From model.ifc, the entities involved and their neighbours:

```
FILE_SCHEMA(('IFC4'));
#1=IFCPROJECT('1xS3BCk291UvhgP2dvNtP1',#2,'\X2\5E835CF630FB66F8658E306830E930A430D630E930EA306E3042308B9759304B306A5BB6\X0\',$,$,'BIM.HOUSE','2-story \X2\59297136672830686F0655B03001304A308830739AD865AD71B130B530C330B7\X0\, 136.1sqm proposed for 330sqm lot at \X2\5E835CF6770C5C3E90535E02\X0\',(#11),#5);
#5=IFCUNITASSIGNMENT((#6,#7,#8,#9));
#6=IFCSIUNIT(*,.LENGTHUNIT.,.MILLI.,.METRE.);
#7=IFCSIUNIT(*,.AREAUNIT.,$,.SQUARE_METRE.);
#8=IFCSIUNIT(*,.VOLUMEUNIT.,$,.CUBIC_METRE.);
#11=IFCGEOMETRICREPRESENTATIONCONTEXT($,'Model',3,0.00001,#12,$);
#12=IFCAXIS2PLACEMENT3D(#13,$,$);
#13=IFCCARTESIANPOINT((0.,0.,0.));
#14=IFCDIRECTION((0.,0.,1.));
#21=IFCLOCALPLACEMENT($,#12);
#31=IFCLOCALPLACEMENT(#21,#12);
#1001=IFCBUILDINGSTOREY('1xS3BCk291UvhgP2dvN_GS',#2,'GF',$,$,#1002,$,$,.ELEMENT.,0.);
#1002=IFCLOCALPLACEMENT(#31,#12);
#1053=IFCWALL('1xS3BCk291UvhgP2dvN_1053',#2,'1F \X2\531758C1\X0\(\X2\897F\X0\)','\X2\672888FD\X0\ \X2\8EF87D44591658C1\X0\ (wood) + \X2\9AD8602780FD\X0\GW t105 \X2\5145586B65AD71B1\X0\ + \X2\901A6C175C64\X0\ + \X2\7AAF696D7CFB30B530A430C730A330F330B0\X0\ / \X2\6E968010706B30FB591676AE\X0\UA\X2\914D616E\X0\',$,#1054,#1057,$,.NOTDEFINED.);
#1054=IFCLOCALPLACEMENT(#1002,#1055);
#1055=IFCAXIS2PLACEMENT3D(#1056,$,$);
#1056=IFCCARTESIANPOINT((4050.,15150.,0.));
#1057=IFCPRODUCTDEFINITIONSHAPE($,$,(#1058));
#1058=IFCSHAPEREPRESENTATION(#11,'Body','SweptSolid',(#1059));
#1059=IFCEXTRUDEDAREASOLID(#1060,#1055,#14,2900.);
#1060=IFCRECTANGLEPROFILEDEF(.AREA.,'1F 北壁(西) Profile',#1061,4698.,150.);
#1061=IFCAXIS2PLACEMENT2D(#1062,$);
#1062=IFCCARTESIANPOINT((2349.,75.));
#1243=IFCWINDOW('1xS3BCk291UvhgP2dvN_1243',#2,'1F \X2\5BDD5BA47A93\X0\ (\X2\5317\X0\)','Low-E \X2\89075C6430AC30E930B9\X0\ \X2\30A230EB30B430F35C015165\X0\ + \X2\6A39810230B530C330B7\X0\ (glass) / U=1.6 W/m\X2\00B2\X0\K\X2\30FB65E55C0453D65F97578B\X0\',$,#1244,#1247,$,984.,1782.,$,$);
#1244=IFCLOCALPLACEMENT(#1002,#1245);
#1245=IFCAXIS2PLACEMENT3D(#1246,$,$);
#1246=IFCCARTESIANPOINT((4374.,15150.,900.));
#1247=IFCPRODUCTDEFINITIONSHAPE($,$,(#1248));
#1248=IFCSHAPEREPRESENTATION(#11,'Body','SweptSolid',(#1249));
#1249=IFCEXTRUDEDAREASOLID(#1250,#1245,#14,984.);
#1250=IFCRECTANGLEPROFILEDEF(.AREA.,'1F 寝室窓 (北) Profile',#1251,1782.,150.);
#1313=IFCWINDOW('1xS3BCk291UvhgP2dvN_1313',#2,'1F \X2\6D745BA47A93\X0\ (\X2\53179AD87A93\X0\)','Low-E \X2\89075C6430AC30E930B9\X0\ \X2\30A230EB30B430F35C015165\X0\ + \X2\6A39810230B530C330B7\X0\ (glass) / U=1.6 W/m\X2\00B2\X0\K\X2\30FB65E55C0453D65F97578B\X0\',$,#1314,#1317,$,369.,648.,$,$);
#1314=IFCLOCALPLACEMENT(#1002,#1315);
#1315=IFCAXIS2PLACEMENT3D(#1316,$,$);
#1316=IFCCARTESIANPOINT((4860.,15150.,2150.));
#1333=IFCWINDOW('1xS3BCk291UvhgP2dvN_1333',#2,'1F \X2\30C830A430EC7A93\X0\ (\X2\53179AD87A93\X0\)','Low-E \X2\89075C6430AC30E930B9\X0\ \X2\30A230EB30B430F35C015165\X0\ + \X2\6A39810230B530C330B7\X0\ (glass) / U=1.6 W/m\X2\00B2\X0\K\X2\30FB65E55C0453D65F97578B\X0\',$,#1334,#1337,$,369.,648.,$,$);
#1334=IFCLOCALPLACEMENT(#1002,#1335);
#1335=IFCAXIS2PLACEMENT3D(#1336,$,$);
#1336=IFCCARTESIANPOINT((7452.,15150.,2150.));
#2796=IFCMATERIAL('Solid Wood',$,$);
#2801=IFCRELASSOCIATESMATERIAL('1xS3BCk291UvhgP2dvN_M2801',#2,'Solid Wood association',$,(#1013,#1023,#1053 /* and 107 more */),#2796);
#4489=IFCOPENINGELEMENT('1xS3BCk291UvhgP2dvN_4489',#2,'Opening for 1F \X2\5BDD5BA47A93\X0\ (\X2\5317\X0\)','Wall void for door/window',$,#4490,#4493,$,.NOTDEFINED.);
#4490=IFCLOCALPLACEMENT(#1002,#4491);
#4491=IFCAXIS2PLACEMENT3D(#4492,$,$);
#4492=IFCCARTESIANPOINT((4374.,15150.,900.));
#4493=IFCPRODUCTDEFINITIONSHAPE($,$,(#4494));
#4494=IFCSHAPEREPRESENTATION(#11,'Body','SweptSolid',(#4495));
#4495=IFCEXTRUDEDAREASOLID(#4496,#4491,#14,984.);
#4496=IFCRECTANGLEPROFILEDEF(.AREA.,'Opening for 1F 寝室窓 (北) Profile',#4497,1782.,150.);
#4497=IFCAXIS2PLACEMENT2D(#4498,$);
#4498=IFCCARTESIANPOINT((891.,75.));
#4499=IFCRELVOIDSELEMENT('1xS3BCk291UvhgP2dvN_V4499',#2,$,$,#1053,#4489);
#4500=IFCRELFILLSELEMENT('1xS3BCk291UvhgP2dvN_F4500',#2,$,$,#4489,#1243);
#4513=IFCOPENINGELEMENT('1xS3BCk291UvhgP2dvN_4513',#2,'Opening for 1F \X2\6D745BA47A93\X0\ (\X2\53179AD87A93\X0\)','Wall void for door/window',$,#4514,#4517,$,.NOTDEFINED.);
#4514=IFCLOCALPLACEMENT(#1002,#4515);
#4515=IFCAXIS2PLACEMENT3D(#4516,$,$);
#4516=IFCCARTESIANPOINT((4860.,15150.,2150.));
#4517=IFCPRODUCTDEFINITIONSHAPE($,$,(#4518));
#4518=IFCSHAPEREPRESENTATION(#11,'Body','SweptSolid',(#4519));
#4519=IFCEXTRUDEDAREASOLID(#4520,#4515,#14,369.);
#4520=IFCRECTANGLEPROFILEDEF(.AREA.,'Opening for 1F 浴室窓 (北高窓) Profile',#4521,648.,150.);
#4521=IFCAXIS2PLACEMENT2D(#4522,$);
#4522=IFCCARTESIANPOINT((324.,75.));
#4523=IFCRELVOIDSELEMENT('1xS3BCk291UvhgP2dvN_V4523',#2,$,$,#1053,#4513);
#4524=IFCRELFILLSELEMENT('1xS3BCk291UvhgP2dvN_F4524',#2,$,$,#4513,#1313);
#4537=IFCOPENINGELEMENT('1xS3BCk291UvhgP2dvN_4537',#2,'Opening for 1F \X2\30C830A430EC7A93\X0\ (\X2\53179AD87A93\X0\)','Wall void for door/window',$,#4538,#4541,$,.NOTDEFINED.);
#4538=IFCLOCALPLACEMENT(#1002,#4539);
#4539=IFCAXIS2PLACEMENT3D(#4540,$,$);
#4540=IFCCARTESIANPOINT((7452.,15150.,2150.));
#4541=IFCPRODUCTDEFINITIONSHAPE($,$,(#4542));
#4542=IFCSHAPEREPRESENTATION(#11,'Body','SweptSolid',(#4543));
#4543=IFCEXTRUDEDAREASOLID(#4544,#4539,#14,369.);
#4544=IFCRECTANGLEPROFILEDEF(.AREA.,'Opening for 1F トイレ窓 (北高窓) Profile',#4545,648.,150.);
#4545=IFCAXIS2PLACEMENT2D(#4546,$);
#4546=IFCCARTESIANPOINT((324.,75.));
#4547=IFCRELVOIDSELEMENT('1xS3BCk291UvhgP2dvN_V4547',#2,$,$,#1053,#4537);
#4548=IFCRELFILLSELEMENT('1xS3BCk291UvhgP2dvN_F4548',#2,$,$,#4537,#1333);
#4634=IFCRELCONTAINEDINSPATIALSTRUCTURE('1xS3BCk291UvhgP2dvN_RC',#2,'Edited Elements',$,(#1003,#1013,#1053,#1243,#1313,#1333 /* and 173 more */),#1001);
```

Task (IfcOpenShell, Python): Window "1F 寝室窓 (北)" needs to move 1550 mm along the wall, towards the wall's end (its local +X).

```python
import ifcopenshell
import ifcopenshell.api.geometry
import ifcopenshell.util.placement
import ifcopenshell.util.unit

model = ifcopenshell.open("model.ifc")
unit_scale = ifcopenshell.util.unit.calculate_unit_scale(model)

window = model.by_guid("1xS3BCk291UvhgP2dvN_1243")
opening = window.FillsVoids[0].RelatingOpeningElement
wall = opening.VoidsElements[0].RelatingBuildingElement

wall_matrix = ifcopenshell.util.placement.get_local_placement(wall.ObjectPlacement)
shift = wall_matrix[:3, 0] * 1.55 / unit_scale
before = ifcopenshell.util.placement.get_local_placement(window.ObjectPlacement)[:3, 3].copy()

# The window is not placed relative to its opening, so move both.
for product in (opening, window):
    matrix = ifcopenshell.util.placement.get_local_placement(product.ObjectPlacement)
    matrix[:3, 3] += shift
    ifcopenshell.api.geometry.edit_object_placement(model, product=product, matrix=matrix, is_si=False)

after = ifcopenshell.util.placement.get_local_placement(window.ObjectPlacement)[:3, 3]
print("window moved by", (after - before).round(3) + 0.0)

model.write("model_v2.ifc")
```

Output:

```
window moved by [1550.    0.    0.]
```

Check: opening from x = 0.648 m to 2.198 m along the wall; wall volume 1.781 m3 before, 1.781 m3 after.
